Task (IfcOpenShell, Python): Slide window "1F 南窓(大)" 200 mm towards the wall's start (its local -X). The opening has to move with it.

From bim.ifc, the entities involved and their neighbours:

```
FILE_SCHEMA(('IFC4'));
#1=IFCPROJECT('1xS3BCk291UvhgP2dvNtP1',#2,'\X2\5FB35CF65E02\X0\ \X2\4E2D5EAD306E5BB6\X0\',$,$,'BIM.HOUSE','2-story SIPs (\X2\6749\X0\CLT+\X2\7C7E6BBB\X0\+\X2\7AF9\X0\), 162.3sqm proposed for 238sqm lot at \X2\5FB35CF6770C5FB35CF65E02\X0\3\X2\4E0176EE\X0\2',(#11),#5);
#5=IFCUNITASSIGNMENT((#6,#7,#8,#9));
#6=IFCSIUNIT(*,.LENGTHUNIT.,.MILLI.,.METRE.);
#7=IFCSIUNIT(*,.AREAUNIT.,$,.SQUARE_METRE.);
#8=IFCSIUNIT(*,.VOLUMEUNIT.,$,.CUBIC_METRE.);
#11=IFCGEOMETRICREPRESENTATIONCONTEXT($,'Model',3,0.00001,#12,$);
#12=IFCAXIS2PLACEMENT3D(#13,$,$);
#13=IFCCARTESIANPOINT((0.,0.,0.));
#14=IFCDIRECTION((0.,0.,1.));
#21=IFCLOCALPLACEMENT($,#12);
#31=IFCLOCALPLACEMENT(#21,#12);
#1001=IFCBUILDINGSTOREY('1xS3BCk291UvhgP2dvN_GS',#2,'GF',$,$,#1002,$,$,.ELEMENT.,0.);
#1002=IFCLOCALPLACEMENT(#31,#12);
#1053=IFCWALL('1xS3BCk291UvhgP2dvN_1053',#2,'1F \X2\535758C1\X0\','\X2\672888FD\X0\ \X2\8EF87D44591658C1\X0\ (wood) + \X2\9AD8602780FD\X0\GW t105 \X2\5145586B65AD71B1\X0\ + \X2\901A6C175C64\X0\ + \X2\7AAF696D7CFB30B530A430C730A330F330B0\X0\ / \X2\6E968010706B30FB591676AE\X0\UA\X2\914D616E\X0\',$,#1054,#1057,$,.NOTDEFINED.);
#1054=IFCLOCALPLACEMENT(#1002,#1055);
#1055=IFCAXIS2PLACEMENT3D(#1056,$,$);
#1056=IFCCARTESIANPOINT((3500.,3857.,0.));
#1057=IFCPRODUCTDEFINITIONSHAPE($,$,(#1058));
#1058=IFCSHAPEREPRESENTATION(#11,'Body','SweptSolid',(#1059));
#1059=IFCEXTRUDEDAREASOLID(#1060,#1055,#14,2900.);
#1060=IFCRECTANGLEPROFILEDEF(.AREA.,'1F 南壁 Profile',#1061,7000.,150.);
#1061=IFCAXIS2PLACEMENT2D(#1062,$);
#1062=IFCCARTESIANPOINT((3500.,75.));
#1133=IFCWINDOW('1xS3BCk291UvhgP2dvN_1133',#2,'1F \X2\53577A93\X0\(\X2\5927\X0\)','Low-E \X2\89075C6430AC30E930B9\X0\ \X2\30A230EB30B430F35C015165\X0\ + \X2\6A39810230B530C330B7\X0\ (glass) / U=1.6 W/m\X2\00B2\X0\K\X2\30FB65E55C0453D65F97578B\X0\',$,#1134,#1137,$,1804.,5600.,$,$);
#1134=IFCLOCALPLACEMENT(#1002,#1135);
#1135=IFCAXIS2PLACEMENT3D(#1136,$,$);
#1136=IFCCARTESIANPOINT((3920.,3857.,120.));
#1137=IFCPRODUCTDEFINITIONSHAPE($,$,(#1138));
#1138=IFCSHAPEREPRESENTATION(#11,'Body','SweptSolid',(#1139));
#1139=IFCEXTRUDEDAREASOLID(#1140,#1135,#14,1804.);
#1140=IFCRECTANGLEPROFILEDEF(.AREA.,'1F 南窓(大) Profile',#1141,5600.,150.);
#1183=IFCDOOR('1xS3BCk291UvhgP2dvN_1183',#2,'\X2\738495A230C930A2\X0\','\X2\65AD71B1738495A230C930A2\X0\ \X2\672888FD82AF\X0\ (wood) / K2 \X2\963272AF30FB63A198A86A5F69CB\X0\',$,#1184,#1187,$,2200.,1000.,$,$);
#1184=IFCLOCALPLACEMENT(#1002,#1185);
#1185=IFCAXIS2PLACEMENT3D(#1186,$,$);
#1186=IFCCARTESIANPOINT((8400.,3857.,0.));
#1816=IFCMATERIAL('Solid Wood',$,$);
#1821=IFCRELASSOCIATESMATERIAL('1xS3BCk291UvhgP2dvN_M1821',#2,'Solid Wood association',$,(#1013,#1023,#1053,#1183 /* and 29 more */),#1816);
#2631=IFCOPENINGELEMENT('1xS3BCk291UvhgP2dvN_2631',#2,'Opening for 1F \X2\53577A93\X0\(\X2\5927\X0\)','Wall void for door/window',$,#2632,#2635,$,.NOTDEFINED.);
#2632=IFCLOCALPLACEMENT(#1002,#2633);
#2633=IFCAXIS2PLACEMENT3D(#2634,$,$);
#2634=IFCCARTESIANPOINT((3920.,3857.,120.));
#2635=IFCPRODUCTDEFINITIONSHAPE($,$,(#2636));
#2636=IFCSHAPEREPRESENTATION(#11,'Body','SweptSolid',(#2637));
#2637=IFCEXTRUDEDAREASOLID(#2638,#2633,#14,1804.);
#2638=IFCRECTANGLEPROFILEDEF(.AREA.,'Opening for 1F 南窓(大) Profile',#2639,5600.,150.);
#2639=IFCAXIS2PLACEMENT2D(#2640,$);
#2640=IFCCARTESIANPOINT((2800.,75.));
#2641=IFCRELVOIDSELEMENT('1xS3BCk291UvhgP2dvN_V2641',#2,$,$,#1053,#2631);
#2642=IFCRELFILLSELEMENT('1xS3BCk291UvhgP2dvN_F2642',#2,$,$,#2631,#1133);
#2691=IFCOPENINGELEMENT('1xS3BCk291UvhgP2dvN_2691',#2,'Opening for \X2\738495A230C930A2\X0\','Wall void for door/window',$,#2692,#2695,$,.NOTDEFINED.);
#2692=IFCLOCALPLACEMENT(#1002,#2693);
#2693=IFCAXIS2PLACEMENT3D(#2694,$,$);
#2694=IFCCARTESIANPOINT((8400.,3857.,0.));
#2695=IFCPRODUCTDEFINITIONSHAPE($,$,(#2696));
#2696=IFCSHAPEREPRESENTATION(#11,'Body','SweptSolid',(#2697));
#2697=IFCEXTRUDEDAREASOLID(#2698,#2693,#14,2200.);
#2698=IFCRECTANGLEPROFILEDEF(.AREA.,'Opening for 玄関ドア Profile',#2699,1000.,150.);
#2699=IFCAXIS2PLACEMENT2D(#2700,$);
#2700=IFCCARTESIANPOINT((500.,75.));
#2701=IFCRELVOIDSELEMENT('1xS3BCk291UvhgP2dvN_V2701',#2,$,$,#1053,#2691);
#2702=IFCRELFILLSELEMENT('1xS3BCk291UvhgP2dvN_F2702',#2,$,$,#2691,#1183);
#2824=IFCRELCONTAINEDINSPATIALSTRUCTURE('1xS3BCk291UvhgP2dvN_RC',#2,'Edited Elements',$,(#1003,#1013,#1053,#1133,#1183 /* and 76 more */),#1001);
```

```python
import ifcopenshell
import ifcopenshell.api.geometry
import ifcopenshell.util.placement
import ifcopenshell.util.unit

model = ifcopenshell.open("bim.ifc")
unit_scale = ifcopenshell.util.unit.calculate_unit_scale(model)

window = model.by_guid("1xS3BCk291UvhgP2dvN_1133")
opening = window.FillsVoids[0].RelatingOpeningElement
wall = opening.VoidsElements[0].RelatingBuildingElement

wall_matrix = ifcopenshell.util.placement.get_local_placement(wall.ObjectPlacement)
shift = wall_matrix[:3, 0] * -0.2 / unit_scale
before = ifcopenshell.util.placement.get_local_placement(window.ObjectPlacement)[:3, 3].copy()

# The window is not placed relative to its opening, so move both.
for product in (opening, window):
    matrix = ifcopenshell.util.placement.get_local_placement(product.ObjectPlacement)
    matrix[:3, 3] += shift
    ifcopenshell.api.geometry.edit_object_placement(model, product=product, matrix=matrix, is_si=False)

after = ifcopenshell.util.placement.get_local_placement(window.ObjectPlacement)[:3, 3]
print("window moved by", (after - before).round(3) + 0.0)

model.write("bim_rev.ifc")
```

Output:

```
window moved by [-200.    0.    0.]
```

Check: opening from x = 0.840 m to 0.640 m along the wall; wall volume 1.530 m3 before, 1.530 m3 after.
